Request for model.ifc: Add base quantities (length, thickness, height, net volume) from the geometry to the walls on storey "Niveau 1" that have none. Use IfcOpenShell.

First a look at what the model holds.

```python
import ifcopenshell
import ifcopenshell.util.element
import ifcopenshell.util.unit

model = ifcopenshell.open("model.ifc")
print(model.schema)
for unit_type in ("LENGTHUNIT", "AREAUNIT", "VOLUMEUNIT"):
    print(unit_type, ifcopenshell.util.unit.calculate_unit_scale(model, unit_type))
storey = next(s for s in model.by_type("IfcBuildingStorey") if s.Name == "Niveau 1")
walls = [e for e in ifcopenshell.util.element.get_decomposition(storey) if e.is_a("IfcWall")]
for e in sorted(walls, key=lambda e: e.id()):
    print(e.id(), e.is_a(), e.Name, list(ifcopenshell.util.element.get_psets(e, qtos_only=True)), sep=" | ")
```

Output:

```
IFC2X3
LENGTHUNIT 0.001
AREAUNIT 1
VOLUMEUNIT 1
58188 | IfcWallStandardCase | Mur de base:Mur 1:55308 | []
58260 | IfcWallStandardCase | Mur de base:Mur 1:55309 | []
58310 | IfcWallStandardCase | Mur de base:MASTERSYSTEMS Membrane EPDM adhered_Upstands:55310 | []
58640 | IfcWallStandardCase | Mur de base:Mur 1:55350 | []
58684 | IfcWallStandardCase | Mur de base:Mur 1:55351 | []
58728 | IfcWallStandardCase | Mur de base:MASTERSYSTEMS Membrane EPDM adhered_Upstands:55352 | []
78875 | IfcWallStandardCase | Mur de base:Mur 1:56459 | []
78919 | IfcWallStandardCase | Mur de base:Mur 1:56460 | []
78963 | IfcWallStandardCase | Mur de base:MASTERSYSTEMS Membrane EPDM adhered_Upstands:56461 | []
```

```python
import ifcopenshell
import ifcopenshell.api.pset
import ifcopenshell.geom
import ifcopenshell.util.element
import ifcopenshell.util.shape
import ifcopenshell.util.unit

model = ifcopenshell.open("model.ifc")
unit_scale = ifcopenshell.util.unit.calculate_unit_scale(model)
volume_scale = ifcopenshell.util.unit.calculate_unit_scale(model, "VOLUMEUNIT")
settings = ifcopenshell.geom.settings()

storey = next(s for s in model.by_type("IfcBuildingStorey") if s.Name == "Niveau 1")
walls = [e for e in ifcopenshell.util.element.get_decomposition(storey) if e.is_a("IfcWall")]

for e in sorted(walls, key=lambda e: e.id()):
    if ifcopenshell.util.element.get_psets(e, qtos_only=True, should_inherit=False):
        continue
    # Geometry comes back in metres, in the element's own axes.
    shape = ifcopenshell.geom.create_shape(settings, e)
    values = {
        "Length": ifcopenshell.util.shape.get_x(shape.geometry) / unit_scale,
        "Width": ifcopenshell.util.shape.get_y(shape.geometry) / unit_scale,
        "Height": ifcopenshell.util.shape.get_z(shape.geometry) / unit_scale,
        "NetVolume": ifcopenshell.util.shape.get_volume(shape.geometry) / volume_scale,
    }
    qto = ifcopenshell.api.pset.add_qto(model, product=e, name="BaseQuantities")
    ifcopenshell.api.pset.edit_qto(model, qto=qto, properties=values)
    print(e.id(), {k: round(v, 3) for k, v in values.items()})

model.write("model_updated.ifc")
```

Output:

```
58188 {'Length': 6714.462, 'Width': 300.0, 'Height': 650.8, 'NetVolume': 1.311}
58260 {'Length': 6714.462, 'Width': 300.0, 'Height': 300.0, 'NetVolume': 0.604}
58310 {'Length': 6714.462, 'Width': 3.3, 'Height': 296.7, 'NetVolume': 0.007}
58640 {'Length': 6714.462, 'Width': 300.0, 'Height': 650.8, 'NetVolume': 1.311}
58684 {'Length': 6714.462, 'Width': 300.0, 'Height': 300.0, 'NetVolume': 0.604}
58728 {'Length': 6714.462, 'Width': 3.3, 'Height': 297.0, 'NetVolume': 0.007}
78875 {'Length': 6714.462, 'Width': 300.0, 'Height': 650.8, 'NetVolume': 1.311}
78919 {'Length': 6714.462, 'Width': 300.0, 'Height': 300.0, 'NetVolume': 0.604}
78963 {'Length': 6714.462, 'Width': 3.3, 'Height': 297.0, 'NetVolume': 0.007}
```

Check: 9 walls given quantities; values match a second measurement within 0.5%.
